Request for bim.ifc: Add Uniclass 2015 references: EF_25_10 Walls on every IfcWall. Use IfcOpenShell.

First a look at what the model holds.

```python
import ifcopenshell

model = ifcopenshell.open("bim.ifc")
print(model.schema)
print("classifications:", [c.Name for c in model.by_type("IfcClassification")])
for ifc_class in ("IfcDoor", "IfcRoof", "IfcStair", "IfcWall", "IfcWindow"):
    print(ifc_class, len(model.by_type(ifc_class)))
```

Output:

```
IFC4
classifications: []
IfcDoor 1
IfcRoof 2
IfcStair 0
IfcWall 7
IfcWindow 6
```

```python
import ifcopenshell
import ifcopenshell.api.classification

model = ifcopenshell.open("bim.ifc")

system = ifcopenshell.api.classification.add_classification(model, classification="Uniclass 2015")

codes = {
    "IfcWall": ("EF_25_10", "Walls"),
}
for ifc_class, (code, name) in codes.items():
    products = model.by_type(ifc_class)
    ifcopenshell.api.classification.add_reference(
        model, products=products, classification=system, identification=code, name=name
    )
    print(code, len(products))

model.write("bim_rev.ifc")
```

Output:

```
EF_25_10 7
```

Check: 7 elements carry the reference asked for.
